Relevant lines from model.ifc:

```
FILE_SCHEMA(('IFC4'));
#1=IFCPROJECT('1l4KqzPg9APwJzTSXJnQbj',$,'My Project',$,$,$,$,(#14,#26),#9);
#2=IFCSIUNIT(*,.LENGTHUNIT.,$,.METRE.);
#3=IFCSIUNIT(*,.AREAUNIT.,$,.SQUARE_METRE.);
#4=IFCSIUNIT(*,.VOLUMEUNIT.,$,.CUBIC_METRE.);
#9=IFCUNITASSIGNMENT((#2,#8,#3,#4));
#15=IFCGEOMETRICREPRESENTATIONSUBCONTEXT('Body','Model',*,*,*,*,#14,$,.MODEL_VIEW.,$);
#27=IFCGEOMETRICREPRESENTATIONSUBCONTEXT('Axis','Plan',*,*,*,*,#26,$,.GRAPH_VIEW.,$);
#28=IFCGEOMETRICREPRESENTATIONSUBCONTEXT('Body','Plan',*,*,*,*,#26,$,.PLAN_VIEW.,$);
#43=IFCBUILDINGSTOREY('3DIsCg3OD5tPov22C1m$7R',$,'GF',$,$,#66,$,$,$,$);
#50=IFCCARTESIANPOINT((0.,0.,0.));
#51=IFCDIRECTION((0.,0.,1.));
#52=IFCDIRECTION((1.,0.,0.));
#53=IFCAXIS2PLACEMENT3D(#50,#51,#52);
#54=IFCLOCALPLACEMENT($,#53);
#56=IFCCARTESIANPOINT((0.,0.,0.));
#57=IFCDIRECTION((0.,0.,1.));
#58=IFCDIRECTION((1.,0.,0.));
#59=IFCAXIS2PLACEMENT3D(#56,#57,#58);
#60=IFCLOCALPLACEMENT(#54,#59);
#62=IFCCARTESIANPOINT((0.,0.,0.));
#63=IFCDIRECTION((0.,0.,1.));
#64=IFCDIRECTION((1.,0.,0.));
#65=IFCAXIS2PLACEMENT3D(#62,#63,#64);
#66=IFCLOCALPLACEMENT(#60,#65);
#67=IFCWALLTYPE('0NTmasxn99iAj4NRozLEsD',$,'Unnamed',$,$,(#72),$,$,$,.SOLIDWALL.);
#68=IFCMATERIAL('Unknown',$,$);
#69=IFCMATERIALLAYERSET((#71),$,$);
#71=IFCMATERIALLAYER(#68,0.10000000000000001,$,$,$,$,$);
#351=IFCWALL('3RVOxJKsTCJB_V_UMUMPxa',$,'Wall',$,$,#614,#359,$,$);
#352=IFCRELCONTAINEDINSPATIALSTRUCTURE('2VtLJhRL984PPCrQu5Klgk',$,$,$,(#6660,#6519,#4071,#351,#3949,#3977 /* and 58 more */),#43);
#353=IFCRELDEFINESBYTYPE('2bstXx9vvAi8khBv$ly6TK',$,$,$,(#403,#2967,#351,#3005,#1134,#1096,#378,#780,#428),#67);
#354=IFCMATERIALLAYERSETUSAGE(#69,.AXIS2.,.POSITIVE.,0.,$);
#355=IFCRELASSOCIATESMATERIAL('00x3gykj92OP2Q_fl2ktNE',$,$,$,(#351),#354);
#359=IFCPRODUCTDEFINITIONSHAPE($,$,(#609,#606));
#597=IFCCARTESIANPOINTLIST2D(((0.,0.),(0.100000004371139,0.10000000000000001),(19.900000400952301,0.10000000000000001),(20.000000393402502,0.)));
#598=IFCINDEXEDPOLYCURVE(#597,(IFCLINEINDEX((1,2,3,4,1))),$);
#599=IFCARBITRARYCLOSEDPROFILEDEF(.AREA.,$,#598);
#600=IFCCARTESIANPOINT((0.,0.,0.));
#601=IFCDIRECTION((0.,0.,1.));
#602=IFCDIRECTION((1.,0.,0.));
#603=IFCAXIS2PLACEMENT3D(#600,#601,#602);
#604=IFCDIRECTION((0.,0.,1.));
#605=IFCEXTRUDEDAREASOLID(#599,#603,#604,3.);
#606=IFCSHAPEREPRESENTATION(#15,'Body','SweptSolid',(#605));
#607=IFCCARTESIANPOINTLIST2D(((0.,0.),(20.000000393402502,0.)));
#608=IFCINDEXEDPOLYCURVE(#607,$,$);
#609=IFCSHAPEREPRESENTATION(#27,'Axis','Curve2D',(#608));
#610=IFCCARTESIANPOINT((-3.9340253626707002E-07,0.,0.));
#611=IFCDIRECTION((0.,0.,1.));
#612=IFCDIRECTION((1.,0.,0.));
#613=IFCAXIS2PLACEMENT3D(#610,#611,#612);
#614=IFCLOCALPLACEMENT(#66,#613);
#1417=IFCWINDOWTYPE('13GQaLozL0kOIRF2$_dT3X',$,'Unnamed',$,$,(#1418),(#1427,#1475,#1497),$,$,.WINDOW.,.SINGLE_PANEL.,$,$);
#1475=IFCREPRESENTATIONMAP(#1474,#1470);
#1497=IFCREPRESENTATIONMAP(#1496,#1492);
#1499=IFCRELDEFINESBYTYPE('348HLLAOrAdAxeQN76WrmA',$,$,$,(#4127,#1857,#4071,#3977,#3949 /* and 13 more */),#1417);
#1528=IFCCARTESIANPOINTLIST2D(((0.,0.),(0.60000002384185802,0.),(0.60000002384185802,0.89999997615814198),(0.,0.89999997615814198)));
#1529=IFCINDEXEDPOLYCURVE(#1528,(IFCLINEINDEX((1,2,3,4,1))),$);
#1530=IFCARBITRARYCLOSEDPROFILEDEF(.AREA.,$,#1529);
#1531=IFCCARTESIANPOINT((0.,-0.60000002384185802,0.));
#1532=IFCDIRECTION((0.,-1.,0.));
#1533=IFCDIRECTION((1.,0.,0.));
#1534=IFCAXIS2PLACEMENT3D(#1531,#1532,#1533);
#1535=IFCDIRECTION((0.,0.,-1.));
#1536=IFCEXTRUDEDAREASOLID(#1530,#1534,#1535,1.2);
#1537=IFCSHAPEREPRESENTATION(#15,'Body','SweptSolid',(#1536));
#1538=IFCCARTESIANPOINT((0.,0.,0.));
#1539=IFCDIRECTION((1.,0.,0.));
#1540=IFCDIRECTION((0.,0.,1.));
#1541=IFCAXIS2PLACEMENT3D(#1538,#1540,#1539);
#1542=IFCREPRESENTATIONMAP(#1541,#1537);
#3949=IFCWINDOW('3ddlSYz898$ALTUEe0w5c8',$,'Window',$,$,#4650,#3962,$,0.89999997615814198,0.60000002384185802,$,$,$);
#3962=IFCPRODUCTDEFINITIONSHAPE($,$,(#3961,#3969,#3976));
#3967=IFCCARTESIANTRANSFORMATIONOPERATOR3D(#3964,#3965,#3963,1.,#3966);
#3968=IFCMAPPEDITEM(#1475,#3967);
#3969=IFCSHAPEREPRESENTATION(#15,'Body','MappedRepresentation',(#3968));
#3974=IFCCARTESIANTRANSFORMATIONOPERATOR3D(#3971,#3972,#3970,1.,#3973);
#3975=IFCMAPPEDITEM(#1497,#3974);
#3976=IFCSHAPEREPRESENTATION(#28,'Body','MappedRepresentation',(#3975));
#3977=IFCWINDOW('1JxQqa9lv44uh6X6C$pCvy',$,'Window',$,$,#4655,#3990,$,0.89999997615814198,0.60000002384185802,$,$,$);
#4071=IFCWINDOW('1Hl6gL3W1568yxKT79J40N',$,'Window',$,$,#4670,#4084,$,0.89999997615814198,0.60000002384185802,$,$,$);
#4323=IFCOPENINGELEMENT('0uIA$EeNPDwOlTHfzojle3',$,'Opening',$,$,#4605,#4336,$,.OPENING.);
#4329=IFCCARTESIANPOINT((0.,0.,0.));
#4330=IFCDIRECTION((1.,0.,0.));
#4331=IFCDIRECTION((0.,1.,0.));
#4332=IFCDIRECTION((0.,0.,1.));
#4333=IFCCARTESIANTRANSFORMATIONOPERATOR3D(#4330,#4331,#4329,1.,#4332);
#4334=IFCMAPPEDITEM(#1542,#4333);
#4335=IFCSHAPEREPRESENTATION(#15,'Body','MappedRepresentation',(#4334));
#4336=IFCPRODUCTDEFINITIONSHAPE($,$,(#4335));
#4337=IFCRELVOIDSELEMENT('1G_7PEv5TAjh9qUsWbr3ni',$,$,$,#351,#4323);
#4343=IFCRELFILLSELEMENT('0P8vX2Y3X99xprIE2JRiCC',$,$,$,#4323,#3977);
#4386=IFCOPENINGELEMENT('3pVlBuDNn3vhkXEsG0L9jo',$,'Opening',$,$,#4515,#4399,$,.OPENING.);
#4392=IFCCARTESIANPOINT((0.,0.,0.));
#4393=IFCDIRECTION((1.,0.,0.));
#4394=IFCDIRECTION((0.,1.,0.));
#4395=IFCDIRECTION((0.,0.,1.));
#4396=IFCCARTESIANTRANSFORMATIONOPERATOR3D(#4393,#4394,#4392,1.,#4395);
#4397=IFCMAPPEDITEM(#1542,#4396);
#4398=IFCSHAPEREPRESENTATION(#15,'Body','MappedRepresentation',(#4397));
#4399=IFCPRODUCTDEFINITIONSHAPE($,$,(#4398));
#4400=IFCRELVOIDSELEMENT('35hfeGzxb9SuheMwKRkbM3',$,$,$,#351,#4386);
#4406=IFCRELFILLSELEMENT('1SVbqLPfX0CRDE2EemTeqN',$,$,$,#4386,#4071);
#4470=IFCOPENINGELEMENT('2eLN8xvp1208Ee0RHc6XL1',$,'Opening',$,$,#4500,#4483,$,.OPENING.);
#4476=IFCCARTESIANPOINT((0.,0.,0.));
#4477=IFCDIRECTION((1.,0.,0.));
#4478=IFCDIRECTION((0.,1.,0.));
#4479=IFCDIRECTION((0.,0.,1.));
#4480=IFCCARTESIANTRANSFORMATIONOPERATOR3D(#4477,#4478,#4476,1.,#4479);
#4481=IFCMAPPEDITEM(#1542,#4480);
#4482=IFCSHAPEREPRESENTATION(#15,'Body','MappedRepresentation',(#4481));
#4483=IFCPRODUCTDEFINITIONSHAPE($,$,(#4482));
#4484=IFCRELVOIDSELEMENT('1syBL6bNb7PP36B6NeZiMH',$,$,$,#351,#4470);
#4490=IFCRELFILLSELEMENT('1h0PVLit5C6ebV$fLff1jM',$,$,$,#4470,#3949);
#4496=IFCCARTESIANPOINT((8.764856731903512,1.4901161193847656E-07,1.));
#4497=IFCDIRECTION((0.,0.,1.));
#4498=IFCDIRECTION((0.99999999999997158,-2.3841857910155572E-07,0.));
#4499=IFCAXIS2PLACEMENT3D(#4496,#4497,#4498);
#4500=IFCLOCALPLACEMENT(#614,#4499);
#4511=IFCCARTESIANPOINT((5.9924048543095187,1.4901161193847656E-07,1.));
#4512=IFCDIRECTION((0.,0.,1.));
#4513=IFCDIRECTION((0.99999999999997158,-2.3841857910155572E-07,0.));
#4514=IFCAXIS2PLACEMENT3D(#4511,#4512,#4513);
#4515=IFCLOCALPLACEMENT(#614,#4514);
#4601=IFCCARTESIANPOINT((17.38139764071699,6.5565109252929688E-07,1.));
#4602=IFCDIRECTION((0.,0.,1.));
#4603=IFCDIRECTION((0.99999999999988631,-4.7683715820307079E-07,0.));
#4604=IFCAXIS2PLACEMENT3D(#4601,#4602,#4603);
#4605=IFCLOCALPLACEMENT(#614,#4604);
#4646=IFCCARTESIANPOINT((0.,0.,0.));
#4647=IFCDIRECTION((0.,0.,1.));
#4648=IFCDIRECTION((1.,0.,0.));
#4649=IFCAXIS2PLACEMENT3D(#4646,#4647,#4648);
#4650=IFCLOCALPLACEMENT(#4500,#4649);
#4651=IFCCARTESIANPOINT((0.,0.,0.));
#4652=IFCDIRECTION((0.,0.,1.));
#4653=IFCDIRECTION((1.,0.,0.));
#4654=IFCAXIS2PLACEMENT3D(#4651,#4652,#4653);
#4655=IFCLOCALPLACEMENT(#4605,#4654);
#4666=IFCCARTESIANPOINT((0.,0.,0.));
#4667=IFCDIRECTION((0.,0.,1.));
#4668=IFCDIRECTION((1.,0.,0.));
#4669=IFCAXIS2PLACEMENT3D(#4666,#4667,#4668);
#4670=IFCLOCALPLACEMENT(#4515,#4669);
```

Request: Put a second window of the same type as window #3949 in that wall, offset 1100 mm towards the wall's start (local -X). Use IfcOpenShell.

```python
import ifcopenshell
import ifcopenshell.api.feature
import ifcopenshell.api.geometry
import ifcopenshell.api.root
import ifcopenshell.geom
import ifcopenshell.util.element
import ifcopenshell.util.placement
import ifcopenshell.util.shape

model = ifcopenshell.open("model.ifc")
settings = ifcopenshell.geom.settings()


def volume(element):
    """Net volume in cubic metres, openings subtracted."""
    shape = ifcopenshell.geom.create_shape(settings, element)
    return ifcopenshell.util.shape.get_volume(shape.geometry)


window = model.by_guid("3ddlSYz898$ALTUEe0w5c8")
opening = window.FillsVoids[0].RelatingOpeningElement
wall = opening.VoidsElements[0].RelatingBuildingElement
before = volume(wall)
shift = ifcopenshell.util.placement.get_local_placement(wall.ObjectPlacement)[:3, 0] * -1.1

# copy_class copies the void relationship, type, container and properties, but no geometry.
new_opening = ifcopenshell.api.root.copy_class(model, product=opening)
new_opening.Representation = ifcopenshell.util.element.copy_deep(
    model, opening.Representation, exclude=["IfcGeometricRepresentationContext", "IfcRepresentationMap"]
)
new_window = ifcopenshell.api.root.copy_class(model, product=window)
new_window.Representation = ifcopenshell.util.element.copy_deep(
    model, window.Representation, exclude=["IfcGeometricRepresentationContext", "IfcRepresentationMap"]
)
ifcopenshell.api.feature.add_filling(model, opening=new_opening, element=new_window)

for old, new in ((opening, new_opening), (window, new_window)):
    matrix = ifcopenshell.util.placement.get_local_placement(old.ObjectPlacement)
    matrix[:3, 3] += shift
    ifcopenshell.api.geometry.edit_object_placement(model, product=new, matrix=matrix, is_si=False)

after = volume(wall)

print(f"wall volume {before:.3f} -> {after:.3f} m3")

model.write("model_rev.ifc")
```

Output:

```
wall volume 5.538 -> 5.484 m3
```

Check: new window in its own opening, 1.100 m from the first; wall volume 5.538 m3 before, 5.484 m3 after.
